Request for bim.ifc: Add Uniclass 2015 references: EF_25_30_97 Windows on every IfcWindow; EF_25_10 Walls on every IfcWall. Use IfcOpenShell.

First a look at what the model holds.

```python
import ifcopenshell

model = ifcopenshell.open("bim.ifc")
print(model.schema)
print("classifications:", [c.Name for c in model.by_type("IfcClassification")])
for ifc_class in ("IfcDoor", "IfcRoof", "IfcStair", "IfcWall", "IfcWindow"):
    print(ifc_class, len(model.by_type(ifc_class)))
```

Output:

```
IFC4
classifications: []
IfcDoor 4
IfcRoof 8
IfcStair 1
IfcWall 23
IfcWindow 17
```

```python
import ifcopenshell
import ifcopenshell.api.classification

model = ifcopenshell.open("bim.ifc")

system = ifcopenshell.api.classification.add_classification(model, classification="Uniclass 2015")

codes = {
    "IfcWindow": ("EF_25_30_97", "Windows"),
    "IfcWall": ("EF_25_10", "Walls"),
}
for ifc_class, (code, name) in codes.items():
    products = model.by_type(ifc_class)
    ifcopenshell.api.classification.add_reference(
        model, products=products, classification=system, identification=code, name=name
    )
    print(code, len(products))

model.write("bim_updated.ifc")
```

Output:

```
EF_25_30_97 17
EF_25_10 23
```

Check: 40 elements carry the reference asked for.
